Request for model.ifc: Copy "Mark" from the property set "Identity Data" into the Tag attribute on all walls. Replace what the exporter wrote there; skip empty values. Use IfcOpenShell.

First a look at what the model holds.

```python
import ifcopenshell
import ifcopenshell.util.element

model = ifcopenshell.open("model.ifc")
print(model.schema)
walls = model.by_type("IfcWall")
print(len(walls), "walls")
for e in walls[:8]:
    source = ifcopenshell.util.element.get_pset(e, "Identity Data", "Mark")
    target = e.Tag
    print(e.id(), repr(source), repr(target), sep=" | ")
```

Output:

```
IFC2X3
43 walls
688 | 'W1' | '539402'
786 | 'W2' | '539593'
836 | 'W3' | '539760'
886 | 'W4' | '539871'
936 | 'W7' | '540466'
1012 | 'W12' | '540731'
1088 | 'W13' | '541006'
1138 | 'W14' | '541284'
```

```python
import ifcopenshell
import ifcopenshell.util.element

model = ifcopenshell.open("model.ifc")

count = 0
for e in model.by_type("IfcWall"):
    value = ifcopenshell.util.element.get_pset(e, "Identity Data", "Mark")
    current = e.Tag
    if not value or not value.strip() or current == value:
        continue
    e.Tag = value
    count += 1

print(count, "walls updated")

model.write("model-out.ifc")
```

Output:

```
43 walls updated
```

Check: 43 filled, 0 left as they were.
